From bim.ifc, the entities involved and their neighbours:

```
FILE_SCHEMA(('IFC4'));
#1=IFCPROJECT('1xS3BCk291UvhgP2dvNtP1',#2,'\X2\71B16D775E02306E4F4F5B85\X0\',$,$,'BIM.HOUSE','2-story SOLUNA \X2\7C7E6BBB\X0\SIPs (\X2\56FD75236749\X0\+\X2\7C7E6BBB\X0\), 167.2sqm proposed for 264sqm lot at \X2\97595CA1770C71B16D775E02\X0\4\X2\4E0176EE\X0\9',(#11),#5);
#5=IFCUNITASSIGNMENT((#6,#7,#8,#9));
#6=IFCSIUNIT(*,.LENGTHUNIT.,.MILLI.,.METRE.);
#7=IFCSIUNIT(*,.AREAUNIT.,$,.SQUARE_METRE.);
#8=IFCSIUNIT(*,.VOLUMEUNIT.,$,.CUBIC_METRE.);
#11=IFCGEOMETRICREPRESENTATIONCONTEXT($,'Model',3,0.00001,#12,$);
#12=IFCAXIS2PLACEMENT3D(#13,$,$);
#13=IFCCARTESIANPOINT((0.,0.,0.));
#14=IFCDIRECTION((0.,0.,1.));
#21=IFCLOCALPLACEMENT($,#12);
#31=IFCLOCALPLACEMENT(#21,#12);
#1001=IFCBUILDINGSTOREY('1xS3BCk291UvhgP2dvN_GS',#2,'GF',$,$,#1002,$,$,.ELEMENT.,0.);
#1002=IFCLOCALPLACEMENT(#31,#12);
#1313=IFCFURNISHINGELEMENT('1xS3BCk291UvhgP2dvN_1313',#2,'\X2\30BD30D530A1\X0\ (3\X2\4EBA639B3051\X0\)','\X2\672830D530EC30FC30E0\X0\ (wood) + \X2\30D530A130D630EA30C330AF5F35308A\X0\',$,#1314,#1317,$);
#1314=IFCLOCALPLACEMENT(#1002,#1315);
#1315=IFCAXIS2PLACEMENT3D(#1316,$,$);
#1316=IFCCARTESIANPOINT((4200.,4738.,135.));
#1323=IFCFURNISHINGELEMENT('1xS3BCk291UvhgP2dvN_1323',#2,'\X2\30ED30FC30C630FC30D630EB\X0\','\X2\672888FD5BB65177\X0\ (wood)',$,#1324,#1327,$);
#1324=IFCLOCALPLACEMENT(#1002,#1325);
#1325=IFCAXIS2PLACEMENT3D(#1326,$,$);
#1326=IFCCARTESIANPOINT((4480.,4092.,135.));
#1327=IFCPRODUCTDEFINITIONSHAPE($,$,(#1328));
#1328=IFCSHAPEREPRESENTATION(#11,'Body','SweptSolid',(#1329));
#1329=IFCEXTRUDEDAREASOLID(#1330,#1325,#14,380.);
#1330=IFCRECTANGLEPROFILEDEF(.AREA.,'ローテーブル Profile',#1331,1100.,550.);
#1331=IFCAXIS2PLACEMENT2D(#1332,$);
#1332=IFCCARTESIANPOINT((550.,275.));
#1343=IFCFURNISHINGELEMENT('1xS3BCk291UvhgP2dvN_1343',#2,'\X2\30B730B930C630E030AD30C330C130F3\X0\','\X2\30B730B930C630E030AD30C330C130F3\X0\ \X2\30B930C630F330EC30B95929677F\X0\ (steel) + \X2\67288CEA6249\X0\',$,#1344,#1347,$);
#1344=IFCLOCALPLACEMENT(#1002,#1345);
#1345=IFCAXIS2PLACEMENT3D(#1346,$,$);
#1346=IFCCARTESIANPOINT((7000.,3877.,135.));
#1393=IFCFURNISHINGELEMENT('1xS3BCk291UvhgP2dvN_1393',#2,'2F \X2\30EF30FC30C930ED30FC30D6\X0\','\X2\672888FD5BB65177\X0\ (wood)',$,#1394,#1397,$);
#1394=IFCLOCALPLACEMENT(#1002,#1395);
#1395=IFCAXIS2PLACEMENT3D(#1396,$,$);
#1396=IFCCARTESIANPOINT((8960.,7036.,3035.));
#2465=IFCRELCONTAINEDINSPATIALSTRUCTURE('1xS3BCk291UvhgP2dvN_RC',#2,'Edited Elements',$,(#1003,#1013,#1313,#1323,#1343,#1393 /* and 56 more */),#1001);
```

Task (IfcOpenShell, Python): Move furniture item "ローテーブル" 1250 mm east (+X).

```python
import ifcopenshell
import ifcopenshell.api.geometry
import ifcopenshell.util.placement
import ifcopenshell.util.unit

model = ifcopenshell.open("bim.ifc")
unit_scale = ifcopenshell.util.unit.calculate_unit_scale(model)

item = model.by_guid("1xS3BCk291UvhgP2dvN_1323")
matrix = ifcopenshell.util.placement.get_local_placement(item.ObjectPlacement)
matrix[0, 3] += 1.25 / unit_scale
ifcopenshell.api.geometry.edit_object_placement(model, product=item, matrix=matrix, is_si=False)

print(ifcopenshell.util.placement.get_local_placement(item.ObjectPlacement).round(3) + 0.0)

model.write("bim_rev.ifc")
```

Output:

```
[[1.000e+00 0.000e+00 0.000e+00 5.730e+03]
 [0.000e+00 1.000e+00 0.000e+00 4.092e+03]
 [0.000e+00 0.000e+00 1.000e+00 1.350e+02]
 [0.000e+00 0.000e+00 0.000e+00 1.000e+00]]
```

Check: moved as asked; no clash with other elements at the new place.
